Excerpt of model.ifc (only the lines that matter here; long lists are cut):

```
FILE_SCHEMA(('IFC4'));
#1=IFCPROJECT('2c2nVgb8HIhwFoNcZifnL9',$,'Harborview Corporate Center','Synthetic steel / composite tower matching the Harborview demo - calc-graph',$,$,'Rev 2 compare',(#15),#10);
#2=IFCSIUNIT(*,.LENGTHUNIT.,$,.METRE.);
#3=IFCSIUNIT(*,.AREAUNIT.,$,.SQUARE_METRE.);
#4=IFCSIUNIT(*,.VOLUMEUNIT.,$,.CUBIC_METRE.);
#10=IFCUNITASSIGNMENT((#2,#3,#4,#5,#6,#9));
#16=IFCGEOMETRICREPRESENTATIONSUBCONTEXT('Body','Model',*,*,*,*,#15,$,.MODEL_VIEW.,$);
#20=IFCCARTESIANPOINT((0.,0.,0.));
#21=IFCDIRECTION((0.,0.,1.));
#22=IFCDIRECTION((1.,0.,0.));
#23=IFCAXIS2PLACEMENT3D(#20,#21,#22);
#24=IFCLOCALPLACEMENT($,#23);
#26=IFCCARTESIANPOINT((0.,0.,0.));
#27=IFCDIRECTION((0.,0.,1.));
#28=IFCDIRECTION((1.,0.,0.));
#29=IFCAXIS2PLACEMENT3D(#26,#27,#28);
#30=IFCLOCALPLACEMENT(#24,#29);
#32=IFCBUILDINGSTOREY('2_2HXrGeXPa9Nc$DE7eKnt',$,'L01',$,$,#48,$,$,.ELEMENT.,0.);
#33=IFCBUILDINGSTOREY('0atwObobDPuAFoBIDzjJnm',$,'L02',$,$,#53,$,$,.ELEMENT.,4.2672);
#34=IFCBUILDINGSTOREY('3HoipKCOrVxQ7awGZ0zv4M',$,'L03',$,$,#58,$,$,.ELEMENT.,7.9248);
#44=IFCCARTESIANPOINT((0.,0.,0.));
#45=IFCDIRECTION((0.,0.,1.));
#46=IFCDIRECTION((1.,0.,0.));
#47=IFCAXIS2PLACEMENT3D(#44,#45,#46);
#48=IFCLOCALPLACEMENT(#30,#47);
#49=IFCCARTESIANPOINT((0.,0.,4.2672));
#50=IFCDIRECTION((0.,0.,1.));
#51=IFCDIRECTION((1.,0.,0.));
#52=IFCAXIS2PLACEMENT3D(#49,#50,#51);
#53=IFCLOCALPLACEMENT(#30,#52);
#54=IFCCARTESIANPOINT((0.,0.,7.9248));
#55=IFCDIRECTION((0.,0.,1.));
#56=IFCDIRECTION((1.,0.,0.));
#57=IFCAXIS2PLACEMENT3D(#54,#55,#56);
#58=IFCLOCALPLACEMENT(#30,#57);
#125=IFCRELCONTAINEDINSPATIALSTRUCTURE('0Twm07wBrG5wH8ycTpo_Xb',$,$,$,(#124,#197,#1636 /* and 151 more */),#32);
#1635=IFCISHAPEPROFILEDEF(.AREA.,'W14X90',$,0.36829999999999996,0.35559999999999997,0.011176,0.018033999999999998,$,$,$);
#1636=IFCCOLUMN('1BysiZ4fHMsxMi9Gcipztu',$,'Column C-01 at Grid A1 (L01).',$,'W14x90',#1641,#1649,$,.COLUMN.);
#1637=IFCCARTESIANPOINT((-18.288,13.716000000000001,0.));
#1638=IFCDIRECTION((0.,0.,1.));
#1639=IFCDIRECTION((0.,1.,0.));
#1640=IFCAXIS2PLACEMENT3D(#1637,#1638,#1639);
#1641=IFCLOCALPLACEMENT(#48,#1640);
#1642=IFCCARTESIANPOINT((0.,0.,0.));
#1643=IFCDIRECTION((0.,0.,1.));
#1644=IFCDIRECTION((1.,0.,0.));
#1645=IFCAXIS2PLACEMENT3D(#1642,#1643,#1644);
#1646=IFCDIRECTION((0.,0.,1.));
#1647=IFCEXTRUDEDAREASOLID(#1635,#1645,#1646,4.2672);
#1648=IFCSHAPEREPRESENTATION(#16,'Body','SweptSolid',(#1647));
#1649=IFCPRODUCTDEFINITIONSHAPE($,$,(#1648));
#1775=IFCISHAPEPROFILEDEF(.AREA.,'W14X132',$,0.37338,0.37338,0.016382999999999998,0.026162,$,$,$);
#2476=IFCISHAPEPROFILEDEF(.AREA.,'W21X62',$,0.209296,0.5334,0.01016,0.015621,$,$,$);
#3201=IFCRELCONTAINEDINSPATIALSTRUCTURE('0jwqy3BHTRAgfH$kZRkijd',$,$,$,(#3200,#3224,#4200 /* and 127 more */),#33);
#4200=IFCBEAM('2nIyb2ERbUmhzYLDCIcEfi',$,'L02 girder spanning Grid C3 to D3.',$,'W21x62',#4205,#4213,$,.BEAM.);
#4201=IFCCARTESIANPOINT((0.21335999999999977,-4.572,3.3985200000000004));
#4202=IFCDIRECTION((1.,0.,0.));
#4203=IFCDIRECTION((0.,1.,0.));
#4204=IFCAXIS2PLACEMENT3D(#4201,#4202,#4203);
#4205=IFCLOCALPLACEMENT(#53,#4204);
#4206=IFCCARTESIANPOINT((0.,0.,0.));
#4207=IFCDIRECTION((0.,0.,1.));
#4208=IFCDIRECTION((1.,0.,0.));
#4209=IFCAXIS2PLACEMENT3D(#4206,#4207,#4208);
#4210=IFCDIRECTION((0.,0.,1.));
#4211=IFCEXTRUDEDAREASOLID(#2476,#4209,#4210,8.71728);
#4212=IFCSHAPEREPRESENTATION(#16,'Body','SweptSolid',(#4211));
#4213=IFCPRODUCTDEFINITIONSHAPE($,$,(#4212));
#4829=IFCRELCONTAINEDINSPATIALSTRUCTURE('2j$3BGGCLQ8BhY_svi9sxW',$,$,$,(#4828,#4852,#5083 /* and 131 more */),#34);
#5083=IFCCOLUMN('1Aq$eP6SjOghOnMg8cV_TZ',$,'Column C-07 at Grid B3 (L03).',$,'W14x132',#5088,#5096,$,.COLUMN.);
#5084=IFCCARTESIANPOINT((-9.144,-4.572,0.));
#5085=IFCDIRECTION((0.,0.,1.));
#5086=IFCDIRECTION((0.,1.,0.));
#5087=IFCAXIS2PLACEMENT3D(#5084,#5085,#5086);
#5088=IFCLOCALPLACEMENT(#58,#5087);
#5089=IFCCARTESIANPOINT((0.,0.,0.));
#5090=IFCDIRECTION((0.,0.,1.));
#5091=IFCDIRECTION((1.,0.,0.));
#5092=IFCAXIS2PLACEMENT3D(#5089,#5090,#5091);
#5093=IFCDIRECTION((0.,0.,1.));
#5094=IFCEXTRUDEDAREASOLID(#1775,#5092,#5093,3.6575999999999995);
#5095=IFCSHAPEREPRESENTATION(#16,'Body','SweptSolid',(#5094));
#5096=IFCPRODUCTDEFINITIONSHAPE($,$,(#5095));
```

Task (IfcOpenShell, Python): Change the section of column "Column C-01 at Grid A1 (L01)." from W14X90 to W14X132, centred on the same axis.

```python
import ifcopenshell
import ifcopenshell.util.element
import ifcopenshell.util.representation

model = ifcopenshell.open("model.ifc")

member = model.by_guid("1BysiZ4fHMsxMi9Gcipztu")
source = next(p for p in model.by_type("IfcIShapeProfileDef") if p.ProfileName == "W14X132")

body = ifcopenshell.util.representation.get_representation(member, "Model", "Body")
solid = body.Items[0]
old_profile = solid.SweptArea

# Copy the section's sizes but keep this member's own profile position.
profile = ifcopenshell.util.element.copy(model, source)
profile.Position = old_profile.Position
solid.SweptArea = profile
if not model.get_total_inverses(old_profile):
    ifcopenshell.util.element.remove_deep2(model, old_profile)

print(solid.SweptArea)

model.write("model_v2.ifc")
```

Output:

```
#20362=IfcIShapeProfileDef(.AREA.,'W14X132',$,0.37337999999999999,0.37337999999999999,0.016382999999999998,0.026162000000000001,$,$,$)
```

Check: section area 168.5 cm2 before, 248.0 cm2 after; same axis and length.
